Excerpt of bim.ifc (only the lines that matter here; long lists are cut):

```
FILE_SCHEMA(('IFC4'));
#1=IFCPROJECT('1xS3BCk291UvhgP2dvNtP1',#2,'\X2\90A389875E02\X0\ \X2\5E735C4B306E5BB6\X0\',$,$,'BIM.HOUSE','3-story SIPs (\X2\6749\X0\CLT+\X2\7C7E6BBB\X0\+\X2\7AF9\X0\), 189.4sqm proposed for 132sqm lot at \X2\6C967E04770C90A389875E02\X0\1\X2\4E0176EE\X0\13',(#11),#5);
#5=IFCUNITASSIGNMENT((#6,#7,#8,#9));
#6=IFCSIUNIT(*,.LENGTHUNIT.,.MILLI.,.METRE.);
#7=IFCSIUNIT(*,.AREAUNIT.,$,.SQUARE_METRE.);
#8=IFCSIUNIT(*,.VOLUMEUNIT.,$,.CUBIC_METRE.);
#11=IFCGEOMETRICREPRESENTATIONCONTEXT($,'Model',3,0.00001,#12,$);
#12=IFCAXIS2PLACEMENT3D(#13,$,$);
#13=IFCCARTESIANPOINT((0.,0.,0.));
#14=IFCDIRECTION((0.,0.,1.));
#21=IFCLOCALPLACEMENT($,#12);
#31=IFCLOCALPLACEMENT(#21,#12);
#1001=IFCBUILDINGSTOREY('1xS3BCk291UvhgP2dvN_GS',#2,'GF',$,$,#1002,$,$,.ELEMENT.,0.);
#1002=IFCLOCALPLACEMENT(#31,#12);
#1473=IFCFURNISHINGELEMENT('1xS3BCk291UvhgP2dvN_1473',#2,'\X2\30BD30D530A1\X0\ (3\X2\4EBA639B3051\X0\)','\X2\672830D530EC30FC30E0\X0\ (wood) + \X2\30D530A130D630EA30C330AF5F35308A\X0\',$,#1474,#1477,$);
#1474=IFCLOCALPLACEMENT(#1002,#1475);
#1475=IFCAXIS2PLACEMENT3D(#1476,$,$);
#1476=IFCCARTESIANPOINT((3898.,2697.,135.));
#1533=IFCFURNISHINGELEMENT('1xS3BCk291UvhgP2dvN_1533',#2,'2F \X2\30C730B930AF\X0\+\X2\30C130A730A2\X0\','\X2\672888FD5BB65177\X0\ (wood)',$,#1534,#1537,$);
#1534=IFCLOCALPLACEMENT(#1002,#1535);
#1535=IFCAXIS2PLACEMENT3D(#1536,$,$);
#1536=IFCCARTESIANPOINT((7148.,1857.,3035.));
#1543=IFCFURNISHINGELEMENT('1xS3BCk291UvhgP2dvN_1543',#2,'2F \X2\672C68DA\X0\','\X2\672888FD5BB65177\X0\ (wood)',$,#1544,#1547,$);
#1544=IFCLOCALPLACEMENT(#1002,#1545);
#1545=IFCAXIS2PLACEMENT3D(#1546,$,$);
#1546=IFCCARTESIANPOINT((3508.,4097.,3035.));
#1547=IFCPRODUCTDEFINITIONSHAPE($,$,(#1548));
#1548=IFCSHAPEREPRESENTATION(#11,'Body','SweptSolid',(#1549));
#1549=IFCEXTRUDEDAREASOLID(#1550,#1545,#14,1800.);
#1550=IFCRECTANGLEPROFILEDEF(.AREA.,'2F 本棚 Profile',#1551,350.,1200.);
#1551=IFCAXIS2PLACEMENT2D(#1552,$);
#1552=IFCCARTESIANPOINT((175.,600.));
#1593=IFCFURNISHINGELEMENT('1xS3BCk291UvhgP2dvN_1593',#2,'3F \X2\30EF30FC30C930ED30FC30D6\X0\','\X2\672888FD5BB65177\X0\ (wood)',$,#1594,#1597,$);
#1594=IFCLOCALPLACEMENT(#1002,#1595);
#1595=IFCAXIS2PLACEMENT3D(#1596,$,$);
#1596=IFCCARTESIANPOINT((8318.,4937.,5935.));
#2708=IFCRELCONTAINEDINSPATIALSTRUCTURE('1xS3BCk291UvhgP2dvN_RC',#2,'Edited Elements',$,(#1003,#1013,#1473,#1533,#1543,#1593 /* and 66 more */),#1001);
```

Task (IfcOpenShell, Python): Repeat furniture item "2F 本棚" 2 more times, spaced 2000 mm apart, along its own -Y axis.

```python
import ifcopenshell
import ifcopenshell.api.geometry
import ifcopenshell.api.root
import ifcopenshell.util.element
import ifcopenshell.util.placement

model = ifcopenshell.open("bim.ifc")


def reuse_history(source, copy):
    """copy_class also copies each property set's owner history, people and application; keep the originals."""
    for rel in copy.IsDefinedBy:
        if rel.is_a("IfcRelDefinesByProperties") and (history := rel.RelatingPropertyDefinition.OwnerHistory):
            rel.RelatingPropertyDefinition.OwnerHistory = source.OwnerHistory
            ifcopenshell.util.element.remove_deep2(model, history)


source = model.by_guid("1xS3BCk291UvhgP2dvN_1543")
base = ifcopenshell.util.placement.get_local_placement(source.ObjectPlacement)
step = -base[:3, 1] * 2000.0

for i in range(1, 3):
    copy = ifcopenshell.api.root.copy_class(model, product=source)
    copy.Representation = ifcopenshell.util.element.copy_deep(
        model, source.Representation, exclude=["IfcGeometricRepresentationContext", "IfcRepresentationMap"]
    )
    reuse_history(source, copy)
    matrix = base.copy()
    matrix[:3, 3] += i * step
    print("added at", matrix[:3, 3].round(3) + 0.0)
    ifcopenshell.api.geometry.edit_object_placement(model, product=copy, matrix=matrix, is_si=False)

model.write("bim_v2.ifc")
```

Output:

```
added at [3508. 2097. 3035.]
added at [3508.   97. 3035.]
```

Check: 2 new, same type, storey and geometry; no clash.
